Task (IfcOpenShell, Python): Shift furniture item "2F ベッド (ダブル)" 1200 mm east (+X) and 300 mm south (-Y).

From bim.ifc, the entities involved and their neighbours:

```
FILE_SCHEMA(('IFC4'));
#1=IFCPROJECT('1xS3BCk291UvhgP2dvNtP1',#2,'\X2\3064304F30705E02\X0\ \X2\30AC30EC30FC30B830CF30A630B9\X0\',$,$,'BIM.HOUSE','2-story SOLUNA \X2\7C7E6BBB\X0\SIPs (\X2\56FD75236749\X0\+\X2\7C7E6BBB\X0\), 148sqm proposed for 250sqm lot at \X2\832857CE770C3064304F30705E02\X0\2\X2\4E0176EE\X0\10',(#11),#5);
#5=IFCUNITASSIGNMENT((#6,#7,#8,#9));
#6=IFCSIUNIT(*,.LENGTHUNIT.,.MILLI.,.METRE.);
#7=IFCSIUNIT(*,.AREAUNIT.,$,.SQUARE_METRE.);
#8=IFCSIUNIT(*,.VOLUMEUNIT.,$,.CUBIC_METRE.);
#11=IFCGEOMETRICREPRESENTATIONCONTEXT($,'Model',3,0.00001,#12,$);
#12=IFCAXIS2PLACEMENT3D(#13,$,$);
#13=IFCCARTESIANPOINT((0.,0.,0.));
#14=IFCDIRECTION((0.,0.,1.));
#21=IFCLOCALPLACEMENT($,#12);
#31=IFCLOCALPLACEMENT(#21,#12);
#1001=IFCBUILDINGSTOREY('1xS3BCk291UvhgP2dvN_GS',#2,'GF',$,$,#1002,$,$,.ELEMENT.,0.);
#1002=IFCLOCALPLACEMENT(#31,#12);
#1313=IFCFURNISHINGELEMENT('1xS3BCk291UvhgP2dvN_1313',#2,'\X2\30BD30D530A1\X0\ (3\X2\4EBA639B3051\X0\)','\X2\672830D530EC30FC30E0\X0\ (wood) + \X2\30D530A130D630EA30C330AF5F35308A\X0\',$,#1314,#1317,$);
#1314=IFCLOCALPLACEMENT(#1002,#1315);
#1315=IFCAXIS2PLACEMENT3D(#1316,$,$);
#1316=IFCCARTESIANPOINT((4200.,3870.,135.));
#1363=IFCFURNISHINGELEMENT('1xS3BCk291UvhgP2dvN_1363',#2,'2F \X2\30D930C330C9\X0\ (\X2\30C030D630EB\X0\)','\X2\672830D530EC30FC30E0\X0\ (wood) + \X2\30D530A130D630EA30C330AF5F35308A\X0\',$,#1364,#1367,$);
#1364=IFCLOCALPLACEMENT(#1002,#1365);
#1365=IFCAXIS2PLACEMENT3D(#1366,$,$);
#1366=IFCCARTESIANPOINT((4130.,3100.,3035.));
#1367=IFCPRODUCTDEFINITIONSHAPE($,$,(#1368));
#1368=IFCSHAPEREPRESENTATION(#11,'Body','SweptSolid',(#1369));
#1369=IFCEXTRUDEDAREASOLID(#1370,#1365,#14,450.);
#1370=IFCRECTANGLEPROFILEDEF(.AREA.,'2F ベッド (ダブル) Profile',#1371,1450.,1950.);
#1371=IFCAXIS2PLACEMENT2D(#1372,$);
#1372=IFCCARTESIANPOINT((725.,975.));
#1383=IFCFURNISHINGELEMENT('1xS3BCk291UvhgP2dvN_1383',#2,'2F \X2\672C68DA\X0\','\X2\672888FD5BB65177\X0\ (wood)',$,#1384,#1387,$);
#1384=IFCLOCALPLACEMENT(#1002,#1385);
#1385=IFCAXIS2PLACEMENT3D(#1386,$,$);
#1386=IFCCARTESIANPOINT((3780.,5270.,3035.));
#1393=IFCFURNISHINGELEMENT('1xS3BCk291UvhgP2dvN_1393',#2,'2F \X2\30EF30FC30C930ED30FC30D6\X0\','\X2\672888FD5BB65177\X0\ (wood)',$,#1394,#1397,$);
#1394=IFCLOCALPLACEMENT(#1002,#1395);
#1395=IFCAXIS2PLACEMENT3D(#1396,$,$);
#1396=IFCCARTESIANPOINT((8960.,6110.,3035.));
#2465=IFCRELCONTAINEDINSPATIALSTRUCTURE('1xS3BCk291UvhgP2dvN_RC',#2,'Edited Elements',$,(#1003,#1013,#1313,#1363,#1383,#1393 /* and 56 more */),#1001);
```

```python
import ifcopenshell
import ifcopenshell.api.geometry
import ifcopenshell.util.placement
import ifcopenshell.util.unit

model = ifcopenshell.open("bim.ifc")
unit_scale = ifcopenshell.util.unit.calculate_unit_scale(model)

item = model.by_guid("1xS3BCk291UvhgP2dvN_1363")
matrix = ifcopenshell.util.placement.get_local_placement(item.ObjectPlacement)
matrix[0, 3] += 1.2 / unit_scale
matrix[1, 3] -= 0.3 / unit_scale
ifcopenshell.api.geometry.edit_object_placement(model, product=item, matrix=matrix, is_si=False)

print(ifcopenshell.util.placement.get_local_placement(item.ObjectPlacement).round(3) + 0.0)

model.write("bim_updated.ifc")
```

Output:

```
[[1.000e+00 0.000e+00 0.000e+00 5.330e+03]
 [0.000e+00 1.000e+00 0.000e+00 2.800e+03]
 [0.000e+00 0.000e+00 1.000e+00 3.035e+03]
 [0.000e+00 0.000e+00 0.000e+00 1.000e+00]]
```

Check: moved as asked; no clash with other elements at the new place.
